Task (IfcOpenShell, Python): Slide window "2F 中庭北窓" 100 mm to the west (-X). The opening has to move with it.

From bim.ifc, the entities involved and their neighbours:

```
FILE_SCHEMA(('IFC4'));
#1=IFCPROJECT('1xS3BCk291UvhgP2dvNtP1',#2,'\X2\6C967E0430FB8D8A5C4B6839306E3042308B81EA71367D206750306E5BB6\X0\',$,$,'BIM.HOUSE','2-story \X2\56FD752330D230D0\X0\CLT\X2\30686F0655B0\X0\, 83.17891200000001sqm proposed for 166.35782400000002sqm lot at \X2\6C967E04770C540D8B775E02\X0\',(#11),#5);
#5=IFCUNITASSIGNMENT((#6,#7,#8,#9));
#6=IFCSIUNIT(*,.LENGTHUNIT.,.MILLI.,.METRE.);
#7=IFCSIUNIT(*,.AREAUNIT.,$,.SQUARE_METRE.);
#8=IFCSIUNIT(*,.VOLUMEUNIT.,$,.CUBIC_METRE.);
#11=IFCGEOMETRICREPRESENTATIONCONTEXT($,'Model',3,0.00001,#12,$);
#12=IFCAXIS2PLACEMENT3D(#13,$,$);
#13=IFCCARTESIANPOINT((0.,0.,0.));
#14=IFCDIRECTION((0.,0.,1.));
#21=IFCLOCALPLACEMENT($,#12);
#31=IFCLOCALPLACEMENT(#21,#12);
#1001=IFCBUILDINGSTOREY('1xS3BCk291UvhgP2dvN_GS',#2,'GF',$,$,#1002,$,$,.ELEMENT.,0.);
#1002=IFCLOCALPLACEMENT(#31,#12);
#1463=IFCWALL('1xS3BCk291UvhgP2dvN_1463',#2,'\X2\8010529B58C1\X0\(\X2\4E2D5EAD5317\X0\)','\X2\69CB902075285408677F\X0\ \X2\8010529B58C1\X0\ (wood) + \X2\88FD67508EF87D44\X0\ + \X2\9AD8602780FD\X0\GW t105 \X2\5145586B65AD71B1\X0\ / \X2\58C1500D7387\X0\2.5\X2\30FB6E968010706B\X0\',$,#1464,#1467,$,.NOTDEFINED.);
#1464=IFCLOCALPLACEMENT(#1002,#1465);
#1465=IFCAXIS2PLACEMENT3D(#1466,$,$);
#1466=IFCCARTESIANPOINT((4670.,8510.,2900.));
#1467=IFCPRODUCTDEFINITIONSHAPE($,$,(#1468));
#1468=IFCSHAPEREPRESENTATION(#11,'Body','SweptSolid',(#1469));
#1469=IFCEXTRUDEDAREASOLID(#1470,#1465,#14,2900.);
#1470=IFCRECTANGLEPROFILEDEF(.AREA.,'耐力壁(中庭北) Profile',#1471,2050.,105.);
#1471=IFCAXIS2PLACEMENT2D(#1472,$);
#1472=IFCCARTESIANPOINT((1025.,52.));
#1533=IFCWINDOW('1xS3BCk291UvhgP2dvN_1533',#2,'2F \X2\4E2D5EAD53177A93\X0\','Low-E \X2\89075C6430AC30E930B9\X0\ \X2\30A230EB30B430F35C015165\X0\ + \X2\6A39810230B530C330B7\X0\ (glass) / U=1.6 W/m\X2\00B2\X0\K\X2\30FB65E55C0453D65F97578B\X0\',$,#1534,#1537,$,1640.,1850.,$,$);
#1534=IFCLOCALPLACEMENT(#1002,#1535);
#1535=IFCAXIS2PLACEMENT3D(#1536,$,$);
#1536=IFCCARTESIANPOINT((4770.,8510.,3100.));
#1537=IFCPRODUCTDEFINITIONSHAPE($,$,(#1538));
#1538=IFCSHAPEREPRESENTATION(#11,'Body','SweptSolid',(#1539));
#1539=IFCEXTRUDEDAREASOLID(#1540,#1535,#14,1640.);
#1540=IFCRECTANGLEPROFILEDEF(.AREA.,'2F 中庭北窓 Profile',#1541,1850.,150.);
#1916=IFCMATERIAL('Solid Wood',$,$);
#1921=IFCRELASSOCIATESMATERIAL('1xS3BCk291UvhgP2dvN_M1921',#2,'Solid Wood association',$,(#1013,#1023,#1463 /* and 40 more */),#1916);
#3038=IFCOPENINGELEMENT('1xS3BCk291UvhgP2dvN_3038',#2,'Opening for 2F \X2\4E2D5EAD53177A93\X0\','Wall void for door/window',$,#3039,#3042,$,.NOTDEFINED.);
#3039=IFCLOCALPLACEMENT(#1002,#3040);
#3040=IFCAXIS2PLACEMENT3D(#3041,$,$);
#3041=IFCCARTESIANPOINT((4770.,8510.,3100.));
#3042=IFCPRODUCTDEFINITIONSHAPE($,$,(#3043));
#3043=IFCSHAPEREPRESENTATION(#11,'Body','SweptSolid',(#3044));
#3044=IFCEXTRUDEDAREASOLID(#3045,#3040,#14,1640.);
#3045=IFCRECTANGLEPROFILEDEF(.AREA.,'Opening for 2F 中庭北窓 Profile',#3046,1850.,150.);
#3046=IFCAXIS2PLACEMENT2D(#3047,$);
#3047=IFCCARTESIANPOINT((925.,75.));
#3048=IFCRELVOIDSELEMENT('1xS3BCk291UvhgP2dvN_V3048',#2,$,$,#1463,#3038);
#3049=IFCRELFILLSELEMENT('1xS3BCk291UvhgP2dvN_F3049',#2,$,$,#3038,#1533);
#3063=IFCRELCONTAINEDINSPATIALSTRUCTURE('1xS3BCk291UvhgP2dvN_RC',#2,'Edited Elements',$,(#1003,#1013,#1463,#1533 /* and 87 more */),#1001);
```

```python
import ifcopenshell
import ifcopenshell.api.geometry
import ifcopenshell.util.placement
import ifcopenshell.util.unit

model = ifcopenshell.open("bim.ifc")
unit_scale = ifcopenshell.util.unit.calculate_unit_scale(model)

window = model.by_guid("1xS3BCk291UvhgP2dvN_1533")
opening = window.FillsVoids[0].RelatingOpeningElement
wall = opening.VoidsElements[0].RelatingBuildingElement

wall_matrix = ifcopenshell.util.placement.get_local_placement(wall.ObjectPlacement)
shift = wall_matrix[:3, 0] * -0.1 / unit_scale
before = ifcopenshell.util.placement.get_local_placement(window.ObjectPlacement)[:3, 3].copy()

# The window is not placed relative to its opening, so move both.
for product in (opening, window):
    matrix = ifcopenshell.util.placement.get_local_placement(product.ObjectPlacement)
    matrix[:3, 3] += shift
    ifcopenshell.api.geometry.edit_object_placement(model, product=product, matrix=matrix, is_si=False)

after = ifcopenshell.util.placement.get_local_placement(window.ObjectPlacement)[:3, 3]
print("window moved by", (after - before).round(3) + 0.0)

model.write("bim_updated.ifc")
```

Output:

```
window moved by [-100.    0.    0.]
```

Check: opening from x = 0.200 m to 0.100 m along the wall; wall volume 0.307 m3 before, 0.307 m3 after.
